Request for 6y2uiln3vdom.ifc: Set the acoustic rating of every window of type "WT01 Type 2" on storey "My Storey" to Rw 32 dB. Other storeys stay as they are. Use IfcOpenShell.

First a look at what the model holds.

```python
import ifcopenshell
import ifcopenshell.util.element

model = ifcopenshell.open("6y2uiln3vdom.ifc")
print(model.schema)
storey = next(s for s in model.by_type("IfcBuildingStorey") if s.Name == "My Storey")
windows = [e for e in ifcopenshell.util.element.get_decomposition(storey) if e.is_a("IfcWindow")]
seen = {}
for e in windows:
    element_type = ifcopenshell.util.element.get_type(e)
    key = (element_type.Name if element_type != e and element_type else None, ifcopenshell.util.element.get_pset(e, "Pset_WindowCommon", "AcousticRating"))
    seen[key] = seen.get(key, 0) + 1
for (name, value), count in sorted(seen.items(), key=str):
    print(count, "x", name, "|", value)
```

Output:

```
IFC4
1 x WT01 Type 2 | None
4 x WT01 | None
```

```python
import ifcopenshell
import ifcopenshell.api.pset
import ifcopenshell.util.element

model = ifcopenshell.open("6y2uiln3vdom.ifc")

storey = next(s for s in model.by_type("IfcBuildingStorey") if s.Name == "My Storey")
windows = [e for e in ifcopenshell.util.element.get_decomposition(storey) if e.is_a("IfcWindow")]

count = 0
for e in windows:
    element_type = ifcopenshell.util.element.get_type(e)
    if element_type in (None, e) or element_type.Name != "WT01 Type 2":
        continue
    # add_pset returns the element's existing set when there is one.
    pset = ifcopenshell.api.pset.add_pset(model, product=e, name="Pset_WindowCommon")
    ifcopenshell.api.pset.edit_pset(model, pset=pset, properties={"AcousticRating": "Rw 32 dB"})
    count += 1

print(count, "windows updated")

model.write("6y2uiln3vdom_rev.ifc")
```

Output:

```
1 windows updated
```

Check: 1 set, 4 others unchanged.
